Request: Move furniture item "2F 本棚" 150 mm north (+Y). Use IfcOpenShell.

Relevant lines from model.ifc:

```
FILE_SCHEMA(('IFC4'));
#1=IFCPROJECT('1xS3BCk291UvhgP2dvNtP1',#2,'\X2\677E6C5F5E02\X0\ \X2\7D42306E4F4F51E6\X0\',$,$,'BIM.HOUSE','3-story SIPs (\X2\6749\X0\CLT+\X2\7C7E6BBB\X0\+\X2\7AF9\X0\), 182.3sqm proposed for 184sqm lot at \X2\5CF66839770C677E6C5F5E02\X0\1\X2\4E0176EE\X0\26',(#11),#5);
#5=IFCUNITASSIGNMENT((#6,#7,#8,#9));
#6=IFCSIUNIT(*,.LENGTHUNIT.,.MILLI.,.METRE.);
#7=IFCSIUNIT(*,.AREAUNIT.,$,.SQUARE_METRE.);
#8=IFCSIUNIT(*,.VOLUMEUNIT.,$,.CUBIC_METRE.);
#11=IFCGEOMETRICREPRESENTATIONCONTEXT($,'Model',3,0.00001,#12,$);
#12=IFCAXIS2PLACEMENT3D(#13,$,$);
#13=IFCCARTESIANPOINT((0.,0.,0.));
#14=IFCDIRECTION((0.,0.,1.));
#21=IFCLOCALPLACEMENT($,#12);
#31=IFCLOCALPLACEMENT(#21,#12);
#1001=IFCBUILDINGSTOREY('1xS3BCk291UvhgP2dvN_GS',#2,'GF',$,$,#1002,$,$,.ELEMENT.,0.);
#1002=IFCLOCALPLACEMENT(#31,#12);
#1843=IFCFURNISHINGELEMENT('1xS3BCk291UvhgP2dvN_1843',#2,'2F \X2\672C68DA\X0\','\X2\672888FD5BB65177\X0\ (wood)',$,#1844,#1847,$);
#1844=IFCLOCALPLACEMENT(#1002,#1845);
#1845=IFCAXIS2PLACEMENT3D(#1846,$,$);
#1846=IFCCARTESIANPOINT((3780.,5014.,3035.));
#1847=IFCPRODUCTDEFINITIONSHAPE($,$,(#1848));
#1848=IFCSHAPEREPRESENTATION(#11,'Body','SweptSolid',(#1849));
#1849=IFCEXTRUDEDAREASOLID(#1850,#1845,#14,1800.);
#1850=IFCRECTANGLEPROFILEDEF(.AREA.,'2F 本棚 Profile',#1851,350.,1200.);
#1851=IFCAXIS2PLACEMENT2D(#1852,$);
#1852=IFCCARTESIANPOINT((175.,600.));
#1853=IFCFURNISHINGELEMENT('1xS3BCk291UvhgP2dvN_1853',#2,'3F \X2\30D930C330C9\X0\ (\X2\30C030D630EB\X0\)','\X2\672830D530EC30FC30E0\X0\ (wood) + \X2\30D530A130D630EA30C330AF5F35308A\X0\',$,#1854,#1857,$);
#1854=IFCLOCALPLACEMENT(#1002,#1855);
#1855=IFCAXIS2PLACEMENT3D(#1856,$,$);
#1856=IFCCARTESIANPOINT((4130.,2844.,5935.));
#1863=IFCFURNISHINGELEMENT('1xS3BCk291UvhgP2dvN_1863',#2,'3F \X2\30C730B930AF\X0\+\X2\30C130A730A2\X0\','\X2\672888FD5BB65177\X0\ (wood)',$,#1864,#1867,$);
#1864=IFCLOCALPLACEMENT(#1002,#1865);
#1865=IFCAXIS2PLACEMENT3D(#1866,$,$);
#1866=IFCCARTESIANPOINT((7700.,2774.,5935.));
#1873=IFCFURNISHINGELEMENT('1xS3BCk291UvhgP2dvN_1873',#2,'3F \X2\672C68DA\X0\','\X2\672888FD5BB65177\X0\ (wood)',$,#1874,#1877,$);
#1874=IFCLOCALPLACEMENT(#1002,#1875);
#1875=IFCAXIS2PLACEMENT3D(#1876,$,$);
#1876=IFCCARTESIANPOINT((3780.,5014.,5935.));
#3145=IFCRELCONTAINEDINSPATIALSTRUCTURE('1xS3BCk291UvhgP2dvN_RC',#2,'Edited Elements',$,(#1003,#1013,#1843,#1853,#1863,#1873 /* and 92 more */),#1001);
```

```python
import ifcopenshell
import ifcopenshell.api.geometry
import ifcopenshell.util.placement
import ifcopenshell.util.unit

model = ifcopenshell.open("model.ifc")
unit_scale = ifcopenshell.util.unit.calculate_unit_scale(model)

item = model.by_id(1843)
matrix = ifcopenshell.util.placement.get_local_placement(item.ObjectPlacement)
matrix[1, 3] += 0.15 / unit_scale
ifcopenshell.api.geometry.edit_object_placement(model, product=item, matrix=matrix, is_si=False)

print(ifcopenshell.util.placement.get_local_placement(item.ObjectPlacement).round(3) + 0.0)

model.write("model-out.ifc")
```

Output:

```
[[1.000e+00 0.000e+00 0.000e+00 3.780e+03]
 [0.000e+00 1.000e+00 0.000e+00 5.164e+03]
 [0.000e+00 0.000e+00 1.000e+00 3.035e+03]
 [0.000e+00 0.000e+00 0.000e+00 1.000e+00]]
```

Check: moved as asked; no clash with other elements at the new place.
